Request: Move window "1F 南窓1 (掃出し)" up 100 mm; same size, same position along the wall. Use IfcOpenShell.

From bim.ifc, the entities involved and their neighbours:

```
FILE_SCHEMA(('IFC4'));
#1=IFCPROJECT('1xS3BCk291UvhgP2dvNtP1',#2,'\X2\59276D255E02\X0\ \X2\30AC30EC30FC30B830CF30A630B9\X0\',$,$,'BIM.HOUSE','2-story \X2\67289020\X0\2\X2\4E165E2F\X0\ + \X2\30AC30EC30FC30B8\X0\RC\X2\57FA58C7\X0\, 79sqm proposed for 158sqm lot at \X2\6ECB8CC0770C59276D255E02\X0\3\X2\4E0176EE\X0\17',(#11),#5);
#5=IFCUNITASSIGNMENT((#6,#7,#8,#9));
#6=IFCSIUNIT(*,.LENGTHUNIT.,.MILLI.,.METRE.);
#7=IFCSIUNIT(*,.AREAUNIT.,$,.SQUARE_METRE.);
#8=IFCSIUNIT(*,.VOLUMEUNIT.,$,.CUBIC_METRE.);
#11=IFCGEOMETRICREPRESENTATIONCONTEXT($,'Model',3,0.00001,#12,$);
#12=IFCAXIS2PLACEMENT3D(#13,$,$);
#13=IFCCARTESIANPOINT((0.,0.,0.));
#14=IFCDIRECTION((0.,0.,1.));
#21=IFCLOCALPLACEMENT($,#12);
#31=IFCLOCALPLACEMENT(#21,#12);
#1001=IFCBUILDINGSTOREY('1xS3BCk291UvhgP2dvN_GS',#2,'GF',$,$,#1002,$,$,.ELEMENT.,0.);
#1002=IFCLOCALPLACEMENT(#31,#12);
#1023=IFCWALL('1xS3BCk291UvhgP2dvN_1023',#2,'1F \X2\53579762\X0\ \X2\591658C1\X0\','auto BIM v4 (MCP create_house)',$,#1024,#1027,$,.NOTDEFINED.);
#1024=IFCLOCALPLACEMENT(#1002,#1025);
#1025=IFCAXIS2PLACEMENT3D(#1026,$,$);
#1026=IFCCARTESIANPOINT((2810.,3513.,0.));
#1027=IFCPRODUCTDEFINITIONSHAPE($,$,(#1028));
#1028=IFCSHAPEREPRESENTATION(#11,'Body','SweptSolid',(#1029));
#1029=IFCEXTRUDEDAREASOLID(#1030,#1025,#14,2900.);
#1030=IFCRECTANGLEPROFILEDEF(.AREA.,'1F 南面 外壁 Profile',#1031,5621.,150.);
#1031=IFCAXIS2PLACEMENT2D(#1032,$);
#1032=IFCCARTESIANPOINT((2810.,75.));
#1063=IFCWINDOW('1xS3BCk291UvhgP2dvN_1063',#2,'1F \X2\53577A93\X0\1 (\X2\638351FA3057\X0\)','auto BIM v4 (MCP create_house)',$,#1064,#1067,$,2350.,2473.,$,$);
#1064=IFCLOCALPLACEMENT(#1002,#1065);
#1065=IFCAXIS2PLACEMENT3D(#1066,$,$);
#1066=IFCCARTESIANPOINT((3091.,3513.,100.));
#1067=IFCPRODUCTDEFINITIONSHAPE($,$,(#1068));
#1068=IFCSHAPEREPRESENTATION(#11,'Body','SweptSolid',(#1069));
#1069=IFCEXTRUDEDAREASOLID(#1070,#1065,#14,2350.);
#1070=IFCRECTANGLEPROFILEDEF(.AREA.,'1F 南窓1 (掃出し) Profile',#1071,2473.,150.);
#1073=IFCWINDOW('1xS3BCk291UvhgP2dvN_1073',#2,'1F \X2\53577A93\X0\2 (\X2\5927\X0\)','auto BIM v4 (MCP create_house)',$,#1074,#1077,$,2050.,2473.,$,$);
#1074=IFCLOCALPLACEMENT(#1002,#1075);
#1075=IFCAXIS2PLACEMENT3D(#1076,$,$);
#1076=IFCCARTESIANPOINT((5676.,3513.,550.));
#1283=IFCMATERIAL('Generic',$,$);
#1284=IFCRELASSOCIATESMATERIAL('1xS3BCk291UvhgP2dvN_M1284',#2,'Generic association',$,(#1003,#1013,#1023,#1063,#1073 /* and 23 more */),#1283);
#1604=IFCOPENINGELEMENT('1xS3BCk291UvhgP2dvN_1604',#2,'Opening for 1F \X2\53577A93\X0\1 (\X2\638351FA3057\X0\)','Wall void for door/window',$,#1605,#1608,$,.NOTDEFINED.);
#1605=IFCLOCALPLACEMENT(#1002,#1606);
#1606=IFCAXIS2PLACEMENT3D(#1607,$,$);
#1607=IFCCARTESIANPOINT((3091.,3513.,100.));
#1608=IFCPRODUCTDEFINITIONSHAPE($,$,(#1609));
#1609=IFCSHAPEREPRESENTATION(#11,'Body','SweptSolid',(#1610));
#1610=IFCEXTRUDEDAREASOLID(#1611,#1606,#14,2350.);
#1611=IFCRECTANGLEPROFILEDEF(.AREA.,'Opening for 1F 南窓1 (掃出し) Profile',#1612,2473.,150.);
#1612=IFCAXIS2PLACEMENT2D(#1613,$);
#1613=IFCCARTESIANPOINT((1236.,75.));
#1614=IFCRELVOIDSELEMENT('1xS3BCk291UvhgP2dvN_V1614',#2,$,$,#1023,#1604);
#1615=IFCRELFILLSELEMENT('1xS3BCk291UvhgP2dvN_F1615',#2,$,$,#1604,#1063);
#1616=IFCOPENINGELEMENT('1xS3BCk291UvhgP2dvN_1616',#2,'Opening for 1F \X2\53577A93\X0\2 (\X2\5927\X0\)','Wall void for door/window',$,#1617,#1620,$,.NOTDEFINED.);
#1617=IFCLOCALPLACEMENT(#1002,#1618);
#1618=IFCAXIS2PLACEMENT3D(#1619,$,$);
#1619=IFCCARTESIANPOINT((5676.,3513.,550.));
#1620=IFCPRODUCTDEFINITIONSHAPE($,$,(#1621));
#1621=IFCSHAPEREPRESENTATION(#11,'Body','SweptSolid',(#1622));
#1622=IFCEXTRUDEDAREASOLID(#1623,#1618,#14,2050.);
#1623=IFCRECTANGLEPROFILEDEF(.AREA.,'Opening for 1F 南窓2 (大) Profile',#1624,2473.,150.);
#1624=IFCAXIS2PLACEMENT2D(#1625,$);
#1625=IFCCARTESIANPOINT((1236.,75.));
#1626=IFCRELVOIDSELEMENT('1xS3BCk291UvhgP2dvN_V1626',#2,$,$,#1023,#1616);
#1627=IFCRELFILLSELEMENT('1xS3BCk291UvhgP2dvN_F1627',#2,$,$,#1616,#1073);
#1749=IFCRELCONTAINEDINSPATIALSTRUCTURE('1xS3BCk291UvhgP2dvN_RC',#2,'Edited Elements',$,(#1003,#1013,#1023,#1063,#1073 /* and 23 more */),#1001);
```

```python
import numpy as np
import ifcopenshell
import ifcopenshell.api.geometry
import ifcopenshell.util.placement
import ifcopenshell.util.unit

model = ifcopenshell.open("bim.ifc")
unit_scale = ifcopenshell.util.unit.calculate_unit_scale(model)

window = model.by_guid("1xS3BCk291UvhgP2dvN_1063")
opening = window.FillsVoids[0].RelatingOpeningElement
dz = 0.1 / unit_scale

shift = np.array([0.0, 0.0, dz])
# The window is not placed relative to its opening, so move both.
for product in (opening, window):
    matrix = ifcopenshell.util.placement.get_local_placement(product.ObjectPlacement)
    matrix[:3, 3] += shift
    ifcopenshell.api.geometry.edit_object_placement(model, product=product, matrix=matrix, is_si=False)

print(f"moved by {dz * unit_scale:+.3f} m")

model.write("bim-out.ifc")
```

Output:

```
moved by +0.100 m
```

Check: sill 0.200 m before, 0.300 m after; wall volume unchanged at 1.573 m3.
